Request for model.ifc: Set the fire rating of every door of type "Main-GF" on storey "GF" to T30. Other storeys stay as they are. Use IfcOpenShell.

First a look at what the model holds.

```python
import ifcopenshell
import ifcopenshell.util.element

model = ifcopenshell.open("model.ifc")
print(model.schema)
storey = next(s for s in model.by_type("IfcBuildingStorey") if s.Name == "GF")
doors = [e for e in ifcopenshell.util.element.get_decomposition(storey) if e.is_a("IfcDoor")]
seen = {}
for e in doors:
    element_type = ifcopenshell.util.element.get_type(e)
    key = (element_type.Name if element_type != e and element_type else None, ifcopenshell.util.element.get_pset(e, "Pset_DoorCommon", "FireRating"))
    seen[key] = seen.get(key, 0) + 1
for (name, value), count in sorted(seen.items(), key=str):
    print(count, "x", name, "|", value)
```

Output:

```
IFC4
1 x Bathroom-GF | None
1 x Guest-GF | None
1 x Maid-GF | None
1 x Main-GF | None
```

```python
import ifcopenshell
import ifcopenshell.api.pset
import ifcopenshell.util.element

model = ifcopenshell.open("model.ifc")

storey = next(s for s in model.by_type("IfcBuildingStorey") if s.Name == "GF")
doors = [e for e in ifcopenshell.util.element.get_decomposition(storey) if e.is_a("IfcDoor")]

count = 0
for e in doors:
    element_type = ifcopenshell.util.element.get_type(e)
    if element_type in (None, e) or element_type.Name != "Main-GF":
        continue
    # add_pset returns the element's existing set when there is one.
    pset = ifcopenshell.api.pset.add_pset(model, product=e, name="Pset_DoorCommon")
    ifcopenshell.api.pset.edit_pset(model, pset=pset, properties={"FireRating": "T30"})
    count += 1

print(count, "doors updated")

model.write("model_updated.ifc")
```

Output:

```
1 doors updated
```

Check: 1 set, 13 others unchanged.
